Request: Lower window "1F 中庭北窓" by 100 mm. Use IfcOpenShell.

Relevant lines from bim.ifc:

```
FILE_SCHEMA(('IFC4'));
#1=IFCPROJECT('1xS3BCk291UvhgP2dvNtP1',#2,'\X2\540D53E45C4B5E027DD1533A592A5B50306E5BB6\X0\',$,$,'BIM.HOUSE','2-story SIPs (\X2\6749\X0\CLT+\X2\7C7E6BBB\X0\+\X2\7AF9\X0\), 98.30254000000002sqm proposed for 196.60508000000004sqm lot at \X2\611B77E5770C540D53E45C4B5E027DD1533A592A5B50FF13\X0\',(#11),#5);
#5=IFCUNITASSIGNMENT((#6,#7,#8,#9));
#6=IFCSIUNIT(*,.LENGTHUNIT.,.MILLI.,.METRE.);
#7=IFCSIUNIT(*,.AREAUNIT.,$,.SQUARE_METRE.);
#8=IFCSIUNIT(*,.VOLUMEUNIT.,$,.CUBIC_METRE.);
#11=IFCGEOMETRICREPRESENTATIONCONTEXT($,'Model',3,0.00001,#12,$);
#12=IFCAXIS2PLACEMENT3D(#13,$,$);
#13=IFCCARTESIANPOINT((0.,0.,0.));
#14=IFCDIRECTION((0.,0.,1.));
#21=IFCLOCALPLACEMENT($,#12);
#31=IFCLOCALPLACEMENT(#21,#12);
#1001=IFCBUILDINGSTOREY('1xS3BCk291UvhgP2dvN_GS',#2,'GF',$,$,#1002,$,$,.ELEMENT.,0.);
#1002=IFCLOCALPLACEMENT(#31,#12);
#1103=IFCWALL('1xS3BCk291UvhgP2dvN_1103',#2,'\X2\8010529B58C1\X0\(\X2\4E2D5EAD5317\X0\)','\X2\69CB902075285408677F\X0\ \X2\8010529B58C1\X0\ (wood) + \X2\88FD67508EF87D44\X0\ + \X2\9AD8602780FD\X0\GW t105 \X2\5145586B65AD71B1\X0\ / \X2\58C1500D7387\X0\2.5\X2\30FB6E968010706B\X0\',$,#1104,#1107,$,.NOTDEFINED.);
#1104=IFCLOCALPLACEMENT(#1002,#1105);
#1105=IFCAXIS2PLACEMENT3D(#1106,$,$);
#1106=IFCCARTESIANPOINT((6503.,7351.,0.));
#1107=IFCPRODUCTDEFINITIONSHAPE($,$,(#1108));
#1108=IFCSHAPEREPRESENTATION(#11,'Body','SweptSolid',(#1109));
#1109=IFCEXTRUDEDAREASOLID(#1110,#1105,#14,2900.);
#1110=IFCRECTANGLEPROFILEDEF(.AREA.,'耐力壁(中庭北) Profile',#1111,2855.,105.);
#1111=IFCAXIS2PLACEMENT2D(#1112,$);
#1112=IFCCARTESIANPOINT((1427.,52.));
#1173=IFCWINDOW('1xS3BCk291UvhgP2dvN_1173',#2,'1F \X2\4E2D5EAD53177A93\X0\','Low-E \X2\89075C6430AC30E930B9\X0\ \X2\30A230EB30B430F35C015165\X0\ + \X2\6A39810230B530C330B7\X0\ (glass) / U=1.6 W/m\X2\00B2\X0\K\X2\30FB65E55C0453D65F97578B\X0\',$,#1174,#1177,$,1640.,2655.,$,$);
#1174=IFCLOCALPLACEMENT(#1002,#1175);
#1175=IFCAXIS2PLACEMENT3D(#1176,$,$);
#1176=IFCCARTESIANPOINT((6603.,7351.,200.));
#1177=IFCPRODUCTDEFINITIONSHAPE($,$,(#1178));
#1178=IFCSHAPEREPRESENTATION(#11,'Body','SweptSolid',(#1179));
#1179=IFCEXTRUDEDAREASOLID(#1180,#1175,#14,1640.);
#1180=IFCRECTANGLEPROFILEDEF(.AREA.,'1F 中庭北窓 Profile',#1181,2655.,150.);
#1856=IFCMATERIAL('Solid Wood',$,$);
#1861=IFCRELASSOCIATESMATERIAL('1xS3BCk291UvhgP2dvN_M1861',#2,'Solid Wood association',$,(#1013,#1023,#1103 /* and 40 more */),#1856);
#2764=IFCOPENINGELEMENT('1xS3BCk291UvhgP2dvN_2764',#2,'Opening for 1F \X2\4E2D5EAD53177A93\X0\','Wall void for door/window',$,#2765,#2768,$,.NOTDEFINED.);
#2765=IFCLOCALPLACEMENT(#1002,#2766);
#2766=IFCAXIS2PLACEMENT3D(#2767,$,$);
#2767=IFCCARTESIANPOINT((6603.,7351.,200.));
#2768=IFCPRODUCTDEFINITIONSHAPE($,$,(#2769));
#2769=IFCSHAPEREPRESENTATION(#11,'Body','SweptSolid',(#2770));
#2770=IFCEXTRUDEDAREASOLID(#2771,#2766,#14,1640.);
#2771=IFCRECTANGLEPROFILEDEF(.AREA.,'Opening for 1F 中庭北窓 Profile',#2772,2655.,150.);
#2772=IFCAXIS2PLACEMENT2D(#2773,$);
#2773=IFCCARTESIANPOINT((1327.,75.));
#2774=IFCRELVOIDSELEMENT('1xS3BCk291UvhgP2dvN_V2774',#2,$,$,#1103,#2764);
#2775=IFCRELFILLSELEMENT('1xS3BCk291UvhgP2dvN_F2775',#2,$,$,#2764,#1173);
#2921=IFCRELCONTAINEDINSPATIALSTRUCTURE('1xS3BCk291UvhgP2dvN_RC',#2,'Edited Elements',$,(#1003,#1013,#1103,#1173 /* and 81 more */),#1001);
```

```python
import numpy as np
import ifcopenshell
import ifcopenshell.api.geometry
import ifcopenshell.util.placement
import ifcopenshell.util.unit

model = ifcopenshell.open("bim.ifc")
unit_scale = ifcopenshell.util.unit.calculate_unit_scale(model)

window = model.by_guid("1xS3BCk291UvhgP2dvN_1173")
opening = window.FillsVoids[0].RelatingOpeningElement
dz = -0.1 / unit_scale

shift = np.array([0.0, 0.0, dz])
# The window is not placed relative to its opening, so move both.
for product in (opening, window):
    matrix = ifcopenshell.util.placement.get_local_placement(product.ObjectPlacement)
    matrix[:3, 3] += shift
    ifcopenshell.api.geometry.edit_object_placement(model, product=product, matrix=matrix, is_si=False)

print(f"moved by {dz * unit_scale:+.3f} m")

model.write("bim_v2.ifc")
```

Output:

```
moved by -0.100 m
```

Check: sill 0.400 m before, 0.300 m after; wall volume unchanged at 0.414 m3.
